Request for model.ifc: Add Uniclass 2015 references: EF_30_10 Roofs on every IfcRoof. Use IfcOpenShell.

First a look at what the model holds.

```python
import ifcopenshell

model = ifcopenshell.open("model.ifc")
print(model.schema)
print("classifications:", [c.Name for c in model.by_type("IfcClassification")])
for ifc_class in ("IfcDoor", "IfcRoof", "IfcStair", "IfcWall", "IfcWindow"):
    print(ifc_class, len(model.by_type(ifc_class)))
```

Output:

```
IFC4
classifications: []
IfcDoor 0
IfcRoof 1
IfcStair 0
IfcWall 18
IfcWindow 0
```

```python
import ifcopenshell
import ifcopenshell.api.classification

model = ifcopenshell.open("model.ifc")

system = ifcopenshell.api.classification.add_classification(model, classification="Uniclass 2015")

codes = {
    "IfcRoof": ("EF_30_10", "Roofs"),
}
for ifc_class, (code, name) in codes.items():
    products = model.by_type(ifc_class)
    ifcopenshell.api.classification.add_reference(
        model, products=products, classification=system, identification=code, name=name
    )
    print(code, len(products))

model.write("model-out.ifc")
```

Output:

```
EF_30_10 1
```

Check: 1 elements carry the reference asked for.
